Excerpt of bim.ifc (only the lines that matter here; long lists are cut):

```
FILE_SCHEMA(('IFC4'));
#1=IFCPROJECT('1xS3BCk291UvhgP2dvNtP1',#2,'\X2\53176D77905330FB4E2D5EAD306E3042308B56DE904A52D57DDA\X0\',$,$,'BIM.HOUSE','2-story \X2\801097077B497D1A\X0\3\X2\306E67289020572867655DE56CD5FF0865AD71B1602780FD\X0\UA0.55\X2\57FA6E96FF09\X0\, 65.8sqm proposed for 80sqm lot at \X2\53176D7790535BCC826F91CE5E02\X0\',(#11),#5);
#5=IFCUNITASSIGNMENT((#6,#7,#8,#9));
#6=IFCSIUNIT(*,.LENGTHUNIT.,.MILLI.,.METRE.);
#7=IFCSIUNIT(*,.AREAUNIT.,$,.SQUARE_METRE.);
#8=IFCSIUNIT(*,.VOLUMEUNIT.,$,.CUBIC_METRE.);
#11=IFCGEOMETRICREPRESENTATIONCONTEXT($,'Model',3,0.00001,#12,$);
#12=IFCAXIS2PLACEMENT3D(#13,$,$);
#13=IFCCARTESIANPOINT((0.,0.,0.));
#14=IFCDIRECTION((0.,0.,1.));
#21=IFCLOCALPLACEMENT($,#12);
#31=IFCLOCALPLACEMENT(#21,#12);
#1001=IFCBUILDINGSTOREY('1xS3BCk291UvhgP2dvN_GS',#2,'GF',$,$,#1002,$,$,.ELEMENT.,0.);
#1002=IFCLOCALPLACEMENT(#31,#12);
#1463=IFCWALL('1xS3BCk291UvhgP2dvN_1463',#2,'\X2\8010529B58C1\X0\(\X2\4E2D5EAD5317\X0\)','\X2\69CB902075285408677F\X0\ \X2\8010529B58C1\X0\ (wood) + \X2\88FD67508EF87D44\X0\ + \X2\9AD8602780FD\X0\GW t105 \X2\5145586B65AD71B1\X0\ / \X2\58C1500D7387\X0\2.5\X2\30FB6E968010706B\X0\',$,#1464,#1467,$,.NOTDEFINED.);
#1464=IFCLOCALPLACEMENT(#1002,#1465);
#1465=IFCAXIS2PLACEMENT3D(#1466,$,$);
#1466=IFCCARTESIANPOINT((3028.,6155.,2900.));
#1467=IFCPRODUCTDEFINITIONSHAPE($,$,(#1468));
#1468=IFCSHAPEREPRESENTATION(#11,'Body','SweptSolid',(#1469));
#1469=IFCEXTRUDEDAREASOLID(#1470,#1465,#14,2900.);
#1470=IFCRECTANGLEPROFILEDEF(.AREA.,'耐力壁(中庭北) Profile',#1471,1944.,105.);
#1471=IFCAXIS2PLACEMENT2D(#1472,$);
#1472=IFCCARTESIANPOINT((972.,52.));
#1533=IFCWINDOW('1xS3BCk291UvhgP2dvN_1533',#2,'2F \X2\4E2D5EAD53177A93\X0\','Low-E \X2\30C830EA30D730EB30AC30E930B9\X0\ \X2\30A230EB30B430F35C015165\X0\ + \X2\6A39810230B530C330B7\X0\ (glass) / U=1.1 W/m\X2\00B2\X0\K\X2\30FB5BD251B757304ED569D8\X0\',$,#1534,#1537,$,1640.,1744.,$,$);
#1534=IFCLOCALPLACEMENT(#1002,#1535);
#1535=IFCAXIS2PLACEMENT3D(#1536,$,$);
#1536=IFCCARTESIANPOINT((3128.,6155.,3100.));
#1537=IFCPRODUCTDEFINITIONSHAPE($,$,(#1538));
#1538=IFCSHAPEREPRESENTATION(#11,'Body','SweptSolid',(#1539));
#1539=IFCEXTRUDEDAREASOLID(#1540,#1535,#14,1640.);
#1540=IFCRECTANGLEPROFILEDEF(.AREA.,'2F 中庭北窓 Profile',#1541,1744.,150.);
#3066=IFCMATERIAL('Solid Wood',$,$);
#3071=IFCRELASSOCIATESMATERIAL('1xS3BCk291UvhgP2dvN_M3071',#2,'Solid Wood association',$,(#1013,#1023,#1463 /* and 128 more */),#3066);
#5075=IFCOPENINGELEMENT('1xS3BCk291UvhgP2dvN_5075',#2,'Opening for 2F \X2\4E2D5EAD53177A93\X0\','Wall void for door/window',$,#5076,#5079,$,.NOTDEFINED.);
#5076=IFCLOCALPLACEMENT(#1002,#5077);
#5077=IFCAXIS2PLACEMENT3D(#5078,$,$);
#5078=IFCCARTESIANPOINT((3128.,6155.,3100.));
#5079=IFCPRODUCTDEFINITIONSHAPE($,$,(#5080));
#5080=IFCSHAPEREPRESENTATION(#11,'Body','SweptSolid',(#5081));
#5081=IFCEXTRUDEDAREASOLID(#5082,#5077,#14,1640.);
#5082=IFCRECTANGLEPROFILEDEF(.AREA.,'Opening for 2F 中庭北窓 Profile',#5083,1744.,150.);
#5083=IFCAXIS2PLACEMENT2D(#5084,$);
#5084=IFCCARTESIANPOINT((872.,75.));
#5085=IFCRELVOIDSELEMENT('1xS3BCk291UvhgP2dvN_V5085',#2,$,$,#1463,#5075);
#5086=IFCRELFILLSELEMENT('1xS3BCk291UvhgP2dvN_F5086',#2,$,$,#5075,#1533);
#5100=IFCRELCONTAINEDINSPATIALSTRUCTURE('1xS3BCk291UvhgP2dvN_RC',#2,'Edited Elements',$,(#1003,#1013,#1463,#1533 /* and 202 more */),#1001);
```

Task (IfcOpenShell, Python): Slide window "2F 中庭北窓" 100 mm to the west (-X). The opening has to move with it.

```python
import ifcopenshell
import ifcopenshell.api.geometry
import ifcopenshell.util.placement

model = ifcopenshell.open("bim.ifc")

window = model.by_id(1533)
opening = window.FillsVoids[0].RelatingOpeningElement
wall = opening.VoidsElements[0].RelatingBuildingElement

wall_matrix = ifcopenshell.util.placement.get_local_placement(wall.ObjectPlacement)
shift = wall_matrix[:3, 0] * -100.0
before = ifcopenshell.util.placement.get_local_placement(window.ObjectPlacement)[:3, 3].copy()

# The window is not placed relative to its opening, so move both.
for product in (opening, window):
    matrix = ifcopenshell.util.placement.get_local_placement(product.ObjectPlacement)
    matrix[:3, 3] += shift
    ifcopenshell.api.geometry.edit_object_placement(model, product=product, matrix=matrix, is_si=False)

after = ifcopenshell.util.placement.get_local_placement(window.ObjectPlacement)[:3, 3]
print("window moved by", (after - before).round(3) + 0.0)

model.write("bim_v2.ifc")
```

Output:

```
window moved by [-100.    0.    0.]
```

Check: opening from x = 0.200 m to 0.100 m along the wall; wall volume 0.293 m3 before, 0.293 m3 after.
